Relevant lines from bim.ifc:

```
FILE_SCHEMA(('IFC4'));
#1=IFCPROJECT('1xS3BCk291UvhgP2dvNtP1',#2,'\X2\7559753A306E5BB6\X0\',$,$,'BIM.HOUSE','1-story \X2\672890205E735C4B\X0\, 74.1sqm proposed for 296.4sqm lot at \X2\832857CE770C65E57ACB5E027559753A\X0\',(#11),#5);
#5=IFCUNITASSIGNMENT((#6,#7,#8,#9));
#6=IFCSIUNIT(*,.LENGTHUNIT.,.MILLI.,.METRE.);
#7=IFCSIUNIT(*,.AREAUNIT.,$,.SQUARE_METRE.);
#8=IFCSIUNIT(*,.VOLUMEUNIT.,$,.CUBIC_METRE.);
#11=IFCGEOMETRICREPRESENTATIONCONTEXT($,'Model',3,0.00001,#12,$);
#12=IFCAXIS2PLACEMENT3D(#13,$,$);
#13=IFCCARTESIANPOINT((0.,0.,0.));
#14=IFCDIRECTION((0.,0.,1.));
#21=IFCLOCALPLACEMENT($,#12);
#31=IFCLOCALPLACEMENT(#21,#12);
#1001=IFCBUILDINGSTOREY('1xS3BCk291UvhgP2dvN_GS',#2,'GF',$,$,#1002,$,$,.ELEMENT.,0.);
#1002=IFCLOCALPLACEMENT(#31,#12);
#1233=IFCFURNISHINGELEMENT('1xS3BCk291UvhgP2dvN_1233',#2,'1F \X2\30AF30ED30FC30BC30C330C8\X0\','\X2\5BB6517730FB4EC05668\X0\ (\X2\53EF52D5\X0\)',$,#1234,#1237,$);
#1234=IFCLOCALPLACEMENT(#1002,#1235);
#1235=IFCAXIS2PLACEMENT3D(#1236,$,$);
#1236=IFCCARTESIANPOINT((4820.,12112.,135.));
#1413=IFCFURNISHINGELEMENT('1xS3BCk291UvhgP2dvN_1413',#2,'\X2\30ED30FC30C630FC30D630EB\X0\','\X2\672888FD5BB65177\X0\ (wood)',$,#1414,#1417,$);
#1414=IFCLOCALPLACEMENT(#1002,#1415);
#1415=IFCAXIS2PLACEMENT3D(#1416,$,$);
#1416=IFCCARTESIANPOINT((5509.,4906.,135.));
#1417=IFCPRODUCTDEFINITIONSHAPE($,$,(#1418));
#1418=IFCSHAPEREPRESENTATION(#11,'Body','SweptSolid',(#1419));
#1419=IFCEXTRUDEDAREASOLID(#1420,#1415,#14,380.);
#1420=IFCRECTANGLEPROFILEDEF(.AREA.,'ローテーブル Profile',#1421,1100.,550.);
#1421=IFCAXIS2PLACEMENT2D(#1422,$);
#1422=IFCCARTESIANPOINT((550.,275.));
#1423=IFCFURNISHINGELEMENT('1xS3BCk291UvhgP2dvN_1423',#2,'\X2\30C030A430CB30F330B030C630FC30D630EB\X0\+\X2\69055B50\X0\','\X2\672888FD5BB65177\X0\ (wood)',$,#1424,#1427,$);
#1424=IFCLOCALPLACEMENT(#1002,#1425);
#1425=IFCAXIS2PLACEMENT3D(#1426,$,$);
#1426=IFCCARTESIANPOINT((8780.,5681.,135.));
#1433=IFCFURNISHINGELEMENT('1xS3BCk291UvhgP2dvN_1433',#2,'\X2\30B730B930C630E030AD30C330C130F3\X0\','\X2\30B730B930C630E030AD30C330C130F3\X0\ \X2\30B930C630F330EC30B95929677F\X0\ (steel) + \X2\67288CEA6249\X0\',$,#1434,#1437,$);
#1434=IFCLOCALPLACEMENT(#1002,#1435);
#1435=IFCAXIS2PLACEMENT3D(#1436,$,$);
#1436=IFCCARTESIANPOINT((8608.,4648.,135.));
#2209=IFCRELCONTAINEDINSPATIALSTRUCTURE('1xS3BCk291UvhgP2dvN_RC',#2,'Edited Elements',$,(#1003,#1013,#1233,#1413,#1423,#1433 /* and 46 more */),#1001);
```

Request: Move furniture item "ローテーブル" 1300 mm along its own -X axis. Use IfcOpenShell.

```python
import ifcopenshell
import ifcopenshell.api.geometry
import ifcopenshell.util.placement
import ifcopenshell.util.unit

model = ifcopenshell.open("bim.ifc")
unit_scale = ifcopenshell.util.unit.calculate_unit_scale(model)

item = model.by_guid("1xS3BCk291UvhgP2dvN_1413")
matrix = ifcopenshell.util.placement.get_local_placement(item.ObjectPlacement)
matrix[:3, 3] -= matrix[:3, 0] * 1.3 / unit_scale
ifcopenshell.api.geometry.edit_object_placement(model, product=item, matrix=matrix, is_si=False)

print(ifcopenshell.util.placement.get_local_placement(item.ObjectPlacement).round(3) + 0.0)

model.write("bim_updated.ifc")
```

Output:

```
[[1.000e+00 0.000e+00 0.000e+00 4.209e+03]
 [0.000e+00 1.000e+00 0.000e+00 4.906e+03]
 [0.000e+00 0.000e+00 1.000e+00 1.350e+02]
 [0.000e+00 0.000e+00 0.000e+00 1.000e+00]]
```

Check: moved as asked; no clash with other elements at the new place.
